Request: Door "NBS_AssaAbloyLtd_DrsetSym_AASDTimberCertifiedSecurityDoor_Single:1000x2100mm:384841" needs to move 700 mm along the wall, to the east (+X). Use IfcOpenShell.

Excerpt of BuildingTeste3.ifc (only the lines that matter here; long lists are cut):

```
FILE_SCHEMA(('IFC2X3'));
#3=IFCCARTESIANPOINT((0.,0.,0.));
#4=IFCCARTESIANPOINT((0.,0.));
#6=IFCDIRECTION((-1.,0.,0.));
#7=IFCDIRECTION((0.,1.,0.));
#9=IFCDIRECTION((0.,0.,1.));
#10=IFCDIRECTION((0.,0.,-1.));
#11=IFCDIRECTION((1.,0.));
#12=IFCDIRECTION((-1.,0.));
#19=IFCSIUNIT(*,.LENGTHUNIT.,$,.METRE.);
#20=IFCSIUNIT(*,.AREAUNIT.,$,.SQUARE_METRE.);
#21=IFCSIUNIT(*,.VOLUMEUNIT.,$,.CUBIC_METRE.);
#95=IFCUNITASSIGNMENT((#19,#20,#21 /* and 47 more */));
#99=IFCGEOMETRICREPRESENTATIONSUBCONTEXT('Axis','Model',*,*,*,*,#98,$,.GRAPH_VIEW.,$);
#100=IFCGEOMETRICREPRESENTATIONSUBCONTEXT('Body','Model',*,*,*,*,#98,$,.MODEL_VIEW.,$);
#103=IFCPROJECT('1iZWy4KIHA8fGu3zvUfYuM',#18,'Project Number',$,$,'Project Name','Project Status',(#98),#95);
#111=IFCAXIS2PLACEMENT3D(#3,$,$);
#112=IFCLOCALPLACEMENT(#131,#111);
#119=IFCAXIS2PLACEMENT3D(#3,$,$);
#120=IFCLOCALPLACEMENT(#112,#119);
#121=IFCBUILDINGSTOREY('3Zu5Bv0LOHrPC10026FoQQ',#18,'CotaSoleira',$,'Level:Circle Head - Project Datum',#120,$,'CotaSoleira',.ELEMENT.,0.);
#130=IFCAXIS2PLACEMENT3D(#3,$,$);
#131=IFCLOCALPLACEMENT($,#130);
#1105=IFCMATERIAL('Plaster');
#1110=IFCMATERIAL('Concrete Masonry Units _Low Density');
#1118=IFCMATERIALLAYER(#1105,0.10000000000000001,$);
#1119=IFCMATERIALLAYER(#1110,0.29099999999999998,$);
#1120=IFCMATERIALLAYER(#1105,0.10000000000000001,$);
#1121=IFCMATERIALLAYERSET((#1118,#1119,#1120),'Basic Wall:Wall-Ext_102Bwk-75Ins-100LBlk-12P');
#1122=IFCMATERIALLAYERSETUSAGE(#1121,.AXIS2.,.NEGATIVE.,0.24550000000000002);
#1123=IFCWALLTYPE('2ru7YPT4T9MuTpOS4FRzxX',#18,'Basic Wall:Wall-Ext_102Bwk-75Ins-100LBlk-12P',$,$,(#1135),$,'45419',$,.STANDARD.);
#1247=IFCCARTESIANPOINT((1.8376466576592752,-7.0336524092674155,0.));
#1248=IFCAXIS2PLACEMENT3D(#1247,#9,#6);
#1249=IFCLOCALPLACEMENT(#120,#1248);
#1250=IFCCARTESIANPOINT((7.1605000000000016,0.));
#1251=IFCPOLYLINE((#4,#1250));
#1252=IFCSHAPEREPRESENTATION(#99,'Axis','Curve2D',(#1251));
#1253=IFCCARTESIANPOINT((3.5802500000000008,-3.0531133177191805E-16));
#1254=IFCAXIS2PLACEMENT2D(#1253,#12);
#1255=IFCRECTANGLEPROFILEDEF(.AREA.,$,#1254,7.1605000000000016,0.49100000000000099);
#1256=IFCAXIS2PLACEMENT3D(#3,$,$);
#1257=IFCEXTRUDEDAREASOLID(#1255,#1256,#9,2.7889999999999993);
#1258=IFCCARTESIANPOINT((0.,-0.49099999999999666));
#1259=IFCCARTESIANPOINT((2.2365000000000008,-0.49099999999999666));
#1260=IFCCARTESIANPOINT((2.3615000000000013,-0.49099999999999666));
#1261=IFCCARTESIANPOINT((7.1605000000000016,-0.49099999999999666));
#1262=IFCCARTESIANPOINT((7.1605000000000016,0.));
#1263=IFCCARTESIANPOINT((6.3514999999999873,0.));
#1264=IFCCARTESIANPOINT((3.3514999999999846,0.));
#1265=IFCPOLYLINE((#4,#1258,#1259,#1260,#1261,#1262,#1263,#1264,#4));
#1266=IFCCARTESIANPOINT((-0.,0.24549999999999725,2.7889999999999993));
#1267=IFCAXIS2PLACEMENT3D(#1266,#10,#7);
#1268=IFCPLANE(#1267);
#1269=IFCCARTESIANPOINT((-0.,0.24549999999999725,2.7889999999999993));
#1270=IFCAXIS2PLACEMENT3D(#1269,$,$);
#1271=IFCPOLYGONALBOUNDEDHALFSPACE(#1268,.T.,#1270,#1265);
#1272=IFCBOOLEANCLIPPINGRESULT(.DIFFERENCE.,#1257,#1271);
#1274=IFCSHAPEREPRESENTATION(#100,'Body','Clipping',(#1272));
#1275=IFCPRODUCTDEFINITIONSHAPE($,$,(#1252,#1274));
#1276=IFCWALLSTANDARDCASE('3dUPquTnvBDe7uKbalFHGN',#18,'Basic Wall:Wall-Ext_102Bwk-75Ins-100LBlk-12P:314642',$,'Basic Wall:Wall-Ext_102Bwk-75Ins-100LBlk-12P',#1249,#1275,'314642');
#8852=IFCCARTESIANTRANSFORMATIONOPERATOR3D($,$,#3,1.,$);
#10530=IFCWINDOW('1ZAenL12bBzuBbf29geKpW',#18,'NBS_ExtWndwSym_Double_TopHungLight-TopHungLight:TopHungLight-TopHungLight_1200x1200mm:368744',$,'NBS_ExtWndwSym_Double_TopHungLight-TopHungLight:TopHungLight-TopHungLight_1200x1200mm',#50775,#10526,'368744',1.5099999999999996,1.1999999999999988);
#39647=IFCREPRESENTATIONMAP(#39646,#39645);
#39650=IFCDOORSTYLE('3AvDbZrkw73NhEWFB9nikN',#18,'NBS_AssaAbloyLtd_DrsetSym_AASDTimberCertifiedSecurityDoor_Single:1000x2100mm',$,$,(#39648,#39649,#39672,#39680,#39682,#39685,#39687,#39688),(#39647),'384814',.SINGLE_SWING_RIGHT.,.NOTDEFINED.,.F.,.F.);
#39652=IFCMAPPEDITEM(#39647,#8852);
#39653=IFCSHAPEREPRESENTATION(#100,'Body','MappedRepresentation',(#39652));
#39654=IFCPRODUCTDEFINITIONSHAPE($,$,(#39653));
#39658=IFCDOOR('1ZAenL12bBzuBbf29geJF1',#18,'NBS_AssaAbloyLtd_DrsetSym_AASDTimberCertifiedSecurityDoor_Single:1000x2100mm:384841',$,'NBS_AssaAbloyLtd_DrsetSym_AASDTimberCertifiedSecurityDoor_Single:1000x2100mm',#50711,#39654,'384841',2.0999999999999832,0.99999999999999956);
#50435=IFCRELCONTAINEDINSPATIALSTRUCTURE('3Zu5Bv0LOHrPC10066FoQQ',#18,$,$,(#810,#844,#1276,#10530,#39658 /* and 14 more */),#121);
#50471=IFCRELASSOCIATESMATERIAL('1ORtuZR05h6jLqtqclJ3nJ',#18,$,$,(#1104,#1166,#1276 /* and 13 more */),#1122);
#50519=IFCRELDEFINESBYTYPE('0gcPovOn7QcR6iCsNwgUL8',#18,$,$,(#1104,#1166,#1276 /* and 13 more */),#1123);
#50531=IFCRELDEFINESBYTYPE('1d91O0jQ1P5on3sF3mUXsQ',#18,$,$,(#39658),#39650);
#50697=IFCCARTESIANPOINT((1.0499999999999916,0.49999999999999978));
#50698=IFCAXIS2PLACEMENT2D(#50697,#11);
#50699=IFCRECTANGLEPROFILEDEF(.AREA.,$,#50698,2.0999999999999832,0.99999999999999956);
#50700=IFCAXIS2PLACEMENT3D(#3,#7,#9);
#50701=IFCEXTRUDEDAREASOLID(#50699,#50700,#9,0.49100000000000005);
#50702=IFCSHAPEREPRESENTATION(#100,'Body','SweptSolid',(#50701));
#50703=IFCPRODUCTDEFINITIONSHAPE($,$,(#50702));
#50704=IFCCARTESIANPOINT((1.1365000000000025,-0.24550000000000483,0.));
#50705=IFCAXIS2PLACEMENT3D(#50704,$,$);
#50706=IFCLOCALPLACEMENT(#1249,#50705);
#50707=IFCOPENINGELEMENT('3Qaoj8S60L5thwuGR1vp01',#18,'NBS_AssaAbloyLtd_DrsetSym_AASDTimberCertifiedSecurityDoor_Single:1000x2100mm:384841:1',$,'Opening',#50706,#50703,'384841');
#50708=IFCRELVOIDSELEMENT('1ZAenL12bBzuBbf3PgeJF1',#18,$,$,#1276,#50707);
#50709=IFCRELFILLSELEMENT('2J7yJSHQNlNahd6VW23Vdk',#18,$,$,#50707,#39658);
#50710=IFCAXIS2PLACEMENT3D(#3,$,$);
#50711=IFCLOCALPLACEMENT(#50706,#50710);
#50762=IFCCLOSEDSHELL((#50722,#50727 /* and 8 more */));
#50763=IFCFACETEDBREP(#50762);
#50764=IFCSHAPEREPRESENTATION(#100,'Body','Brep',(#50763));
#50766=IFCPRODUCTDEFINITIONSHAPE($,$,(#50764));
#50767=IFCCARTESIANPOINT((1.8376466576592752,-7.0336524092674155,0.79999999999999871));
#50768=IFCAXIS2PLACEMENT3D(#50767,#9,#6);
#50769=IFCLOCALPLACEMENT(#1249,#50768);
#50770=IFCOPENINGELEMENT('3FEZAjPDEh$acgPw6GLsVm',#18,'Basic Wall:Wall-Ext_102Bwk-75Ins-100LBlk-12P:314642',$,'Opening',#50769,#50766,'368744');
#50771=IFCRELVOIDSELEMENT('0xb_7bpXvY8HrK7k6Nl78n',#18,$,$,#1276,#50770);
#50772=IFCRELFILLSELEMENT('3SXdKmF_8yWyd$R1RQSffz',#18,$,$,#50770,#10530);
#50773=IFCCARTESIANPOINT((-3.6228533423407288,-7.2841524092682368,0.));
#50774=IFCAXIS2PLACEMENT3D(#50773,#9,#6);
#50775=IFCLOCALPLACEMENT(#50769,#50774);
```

```python
import ifcopenshell
import ifcopenshell.api.geometry
import ifcopenshell.util.placement
import ifcopenshell.util.unit

model = ifcopenshell.open("BuildingTeste3.ifc")
unit_scale = ifcopenshell.util.unit.calculate_unit_scale(model)

door = model.by_id(39658)
opening = door.FillsVoids[0].RelatingOpeningElement
wall = opening.VoidsElements[0].RelatingBuildingElement

wall_matrix = ifcopenshell.util.placement.get_local_placement(wall.ObjectPlacement)
shift = wall_matrix[:3, 0] * -0.7 / unit_scale
before = ifcopenshell.util.placement.get_local_placement(door.ObjectPlacement)[:3, 3].copy()

# The door is placed relative to its opening, so it follows when the opening moves.
matrix = ifcopenshell.util.placement.get_local_placement(opening.ObjectPlacement)
matrix[:3, 3] += shift
ifcopenshell.api.geometry.edit_object_placement(
    model, product=opening, matrix=matrix, is_si=False, should_transform_children=True
)

after = ifcopenshell.util.placement.get_local_placement(door.ObjectPlacement)[:3, 3]
print("door moved by", (after - before).round(3) + 0.0)

model.write("BuildingTeste3_rev.ifc")
```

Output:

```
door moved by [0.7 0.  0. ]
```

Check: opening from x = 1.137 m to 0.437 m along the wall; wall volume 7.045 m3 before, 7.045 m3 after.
